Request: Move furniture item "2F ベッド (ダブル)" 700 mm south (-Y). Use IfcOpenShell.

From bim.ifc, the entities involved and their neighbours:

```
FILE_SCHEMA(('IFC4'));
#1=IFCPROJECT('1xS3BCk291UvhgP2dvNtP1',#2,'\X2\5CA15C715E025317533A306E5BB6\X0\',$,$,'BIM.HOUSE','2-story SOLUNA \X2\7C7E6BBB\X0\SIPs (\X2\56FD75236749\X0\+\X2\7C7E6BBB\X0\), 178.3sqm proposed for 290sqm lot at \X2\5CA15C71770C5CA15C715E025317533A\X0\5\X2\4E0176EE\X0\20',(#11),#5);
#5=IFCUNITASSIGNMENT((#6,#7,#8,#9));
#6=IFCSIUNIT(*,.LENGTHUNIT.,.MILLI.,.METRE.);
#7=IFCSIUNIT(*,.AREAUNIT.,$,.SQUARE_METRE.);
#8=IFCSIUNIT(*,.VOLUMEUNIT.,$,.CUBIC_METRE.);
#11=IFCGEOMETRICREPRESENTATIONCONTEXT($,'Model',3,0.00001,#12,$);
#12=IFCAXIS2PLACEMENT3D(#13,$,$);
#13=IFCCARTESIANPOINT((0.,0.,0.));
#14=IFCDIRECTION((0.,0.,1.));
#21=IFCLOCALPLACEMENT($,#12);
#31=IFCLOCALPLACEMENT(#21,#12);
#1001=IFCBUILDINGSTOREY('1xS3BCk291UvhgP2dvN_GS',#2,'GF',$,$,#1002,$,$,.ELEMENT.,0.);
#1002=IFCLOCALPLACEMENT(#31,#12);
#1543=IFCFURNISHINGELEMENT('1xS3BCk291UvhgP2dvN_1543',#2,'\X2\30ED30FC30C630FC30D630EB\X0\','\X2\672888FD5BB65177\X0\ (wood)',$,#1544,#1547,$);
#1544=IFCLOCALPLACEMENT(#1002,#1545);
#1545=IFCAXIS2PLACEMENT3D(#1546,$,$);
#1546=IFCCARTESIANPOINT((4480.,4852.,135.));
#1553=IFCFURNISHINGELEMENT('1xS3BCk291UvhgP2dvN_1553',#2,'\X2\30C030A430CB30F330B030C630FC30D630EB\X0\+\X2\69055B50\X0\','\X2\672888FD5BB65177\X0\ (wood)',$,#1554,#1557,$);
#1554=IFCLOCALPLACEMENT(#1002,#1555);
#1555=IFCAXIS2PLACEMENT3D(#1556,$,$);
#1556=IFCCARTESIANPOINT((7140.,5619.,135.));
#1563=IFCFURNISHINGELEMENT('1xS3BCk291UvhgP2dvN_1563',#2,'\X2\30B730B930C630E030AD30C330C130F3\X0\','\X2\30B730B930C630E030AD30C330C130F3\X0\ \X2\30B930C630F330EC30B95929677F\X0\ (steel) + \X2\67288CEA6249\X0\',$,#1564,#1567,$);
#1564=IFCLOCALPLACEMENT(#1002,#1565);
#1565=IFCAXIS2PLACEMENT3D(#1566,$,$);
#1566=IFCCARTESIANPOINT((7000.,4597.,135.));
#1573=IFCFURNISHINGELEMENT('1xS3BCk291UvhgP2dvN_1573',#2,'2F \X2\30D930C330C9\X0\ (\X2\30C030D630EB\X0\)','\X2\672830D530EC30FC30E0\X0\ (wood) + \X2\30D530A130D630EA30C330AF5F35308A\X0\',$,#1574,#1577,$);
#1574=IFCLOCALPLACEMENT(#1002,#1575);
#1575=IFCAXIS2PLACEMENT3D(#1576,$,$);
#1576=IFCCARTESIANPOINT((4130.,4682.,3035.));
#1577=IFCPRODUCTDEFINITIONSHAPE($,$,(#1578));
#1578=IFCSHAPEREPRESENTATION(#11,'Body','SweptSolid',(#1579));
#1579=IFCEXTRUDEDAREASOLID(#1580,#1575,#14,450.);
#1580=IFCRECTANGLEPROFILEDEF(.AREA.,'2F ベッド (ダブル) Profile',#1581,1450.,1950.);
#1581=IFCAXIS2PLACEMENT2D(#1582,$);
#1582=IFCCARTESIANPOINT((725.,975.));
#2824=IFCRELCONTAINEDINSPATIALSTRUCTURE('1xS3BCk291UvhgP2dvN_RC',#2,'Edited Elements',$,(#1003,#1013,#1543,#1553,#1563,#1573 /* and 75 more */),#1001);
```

```python
import ifcopenshell
import ifcopenshell.api.geometry
import ifcopenshell.util.placement

model = ifcopenshell.open("bim.ifc")

item = model.by_id(1573)
matrix = ifcopenshell.util.placement.get_local_placement(item.ObjectPlacement)
matrix[1, 3] -= 700.0
ifcopenshell.api.geometry.edit_object_placement(model, product=item, matrix=matrix, is_si=False)

print(ifcopenshell.util.placement.get_local_placement(item.ObjectPlacement).round(3) + 0.0)

model.write("bim_rev.ifc")
```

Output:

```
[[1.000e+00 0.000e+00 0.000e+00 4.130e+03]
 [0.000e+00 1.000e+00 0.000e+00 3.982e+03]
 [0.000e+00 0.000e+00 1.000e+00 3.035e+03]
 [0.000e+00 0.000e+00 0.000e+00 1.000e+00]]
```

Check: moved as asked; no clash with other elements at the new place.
